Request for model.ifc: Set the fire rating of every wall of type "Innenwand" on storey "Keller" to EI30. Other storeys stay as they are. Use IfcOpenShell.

First a look at what the model holds.

```python
import ifcopenshell
import ifcopenshell.util.element

model = ifcopenshell.open("model.ifc")
print(model.schema)
storey = next(s for s in model.by_type("IfcBuildingStorey") if s.Name == "Keller")
walls = [e for e in ifcopenshell.util.element.get_decomposition(storey) if e.is_a("IfcWall")]
seen = {}
for e in walls:
    element_type = ifcopenshell.util.element.get_type(e)
    key = (element_type.Name if element_type != e and element_type else None, ifcopenshell.util.element.get_pset(e, "Pset_WallCommon", "FireRating"))
    seen[key] = seen.get(key, 0) + 1
for (name, value), count in sorted(seen.items(), key=str):
    print(count, "x", name, "|", value)
```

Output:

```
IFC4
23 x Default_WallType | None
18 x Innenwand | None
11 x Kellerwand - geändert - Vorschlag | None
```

```python
import ifcopenshell
import ifcopenshell.api.pset
import ifcopenshell.util.element

model = ifcopenshell.open("model.ifc")

storey = next(s for s in model.by_type("IfcBuildingStorey") if s.Name == "Keller")
walls = [e for e in ifcopenshell.util.element.get_decomposition(storey) if e.is_a("IfcWall")]

count = 0
for e in walls:
    element_type = ifcopenshell.util.element.get_type(e)
    if element_type in (None, e) or element_type.Name != "Innenwand":
        continue
    # add_pset returns the element's existing set when there is one.
    pset = ifcopenshell.api.pset.add_pset(model, product=e, name="Pset_WallCommon")
    ifcopenshell.api.pset.edit_pset(model, pset=pset, properties={"FireRating": "EI30"})
    count += 1

print(count, "walls updated")

model.write("model_edited.ifc")
```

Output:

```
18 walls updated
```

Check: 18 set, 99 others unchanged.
